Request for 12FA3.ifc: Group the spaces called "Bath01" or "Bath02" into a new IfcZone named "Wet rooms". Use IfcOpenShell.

First a look at what the model holds.

```python
import ifcopenshell

model = ifcopenshell.open("12FA3.ifc")
print(model.schema)
seen = {}
for space in model.by_type("IfcSpace"):
    seen[space.Name] = seen.get(space.Name, 0) + 1
for name, count in sorted(seen.items(), key=str):
    print(count, "x", name)
print("zones:", [z.Name for z in model.by_type("IfcZone")][:20])
```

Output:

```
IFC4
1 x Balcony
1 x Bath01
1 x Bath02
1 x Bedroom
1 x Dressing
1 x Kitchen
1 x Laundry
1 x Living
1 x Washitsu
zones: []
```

```python
import ifcopenshell
import ifcopenshell.api.group
import ifcopenshell.api.root

model = ifcopenshell.open("12FA3.ifc")

names = {"Bath01", "Bath02"}
spaces = [s for s in model.by_type("IfcSpace") if s.Name in names]

zone = ifcopenshell.api.root.create_entity(model, ifc_class="IfcZone", name="Wet rooms")
ifcopenshell.api.group.assign_group(model, products=spaces, group=zone)
print(len(spaces), "spaces in", zone.Name)

model.write("12FA3_v2.ifc")
```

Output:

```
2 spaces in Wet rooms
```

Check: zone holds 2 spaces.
